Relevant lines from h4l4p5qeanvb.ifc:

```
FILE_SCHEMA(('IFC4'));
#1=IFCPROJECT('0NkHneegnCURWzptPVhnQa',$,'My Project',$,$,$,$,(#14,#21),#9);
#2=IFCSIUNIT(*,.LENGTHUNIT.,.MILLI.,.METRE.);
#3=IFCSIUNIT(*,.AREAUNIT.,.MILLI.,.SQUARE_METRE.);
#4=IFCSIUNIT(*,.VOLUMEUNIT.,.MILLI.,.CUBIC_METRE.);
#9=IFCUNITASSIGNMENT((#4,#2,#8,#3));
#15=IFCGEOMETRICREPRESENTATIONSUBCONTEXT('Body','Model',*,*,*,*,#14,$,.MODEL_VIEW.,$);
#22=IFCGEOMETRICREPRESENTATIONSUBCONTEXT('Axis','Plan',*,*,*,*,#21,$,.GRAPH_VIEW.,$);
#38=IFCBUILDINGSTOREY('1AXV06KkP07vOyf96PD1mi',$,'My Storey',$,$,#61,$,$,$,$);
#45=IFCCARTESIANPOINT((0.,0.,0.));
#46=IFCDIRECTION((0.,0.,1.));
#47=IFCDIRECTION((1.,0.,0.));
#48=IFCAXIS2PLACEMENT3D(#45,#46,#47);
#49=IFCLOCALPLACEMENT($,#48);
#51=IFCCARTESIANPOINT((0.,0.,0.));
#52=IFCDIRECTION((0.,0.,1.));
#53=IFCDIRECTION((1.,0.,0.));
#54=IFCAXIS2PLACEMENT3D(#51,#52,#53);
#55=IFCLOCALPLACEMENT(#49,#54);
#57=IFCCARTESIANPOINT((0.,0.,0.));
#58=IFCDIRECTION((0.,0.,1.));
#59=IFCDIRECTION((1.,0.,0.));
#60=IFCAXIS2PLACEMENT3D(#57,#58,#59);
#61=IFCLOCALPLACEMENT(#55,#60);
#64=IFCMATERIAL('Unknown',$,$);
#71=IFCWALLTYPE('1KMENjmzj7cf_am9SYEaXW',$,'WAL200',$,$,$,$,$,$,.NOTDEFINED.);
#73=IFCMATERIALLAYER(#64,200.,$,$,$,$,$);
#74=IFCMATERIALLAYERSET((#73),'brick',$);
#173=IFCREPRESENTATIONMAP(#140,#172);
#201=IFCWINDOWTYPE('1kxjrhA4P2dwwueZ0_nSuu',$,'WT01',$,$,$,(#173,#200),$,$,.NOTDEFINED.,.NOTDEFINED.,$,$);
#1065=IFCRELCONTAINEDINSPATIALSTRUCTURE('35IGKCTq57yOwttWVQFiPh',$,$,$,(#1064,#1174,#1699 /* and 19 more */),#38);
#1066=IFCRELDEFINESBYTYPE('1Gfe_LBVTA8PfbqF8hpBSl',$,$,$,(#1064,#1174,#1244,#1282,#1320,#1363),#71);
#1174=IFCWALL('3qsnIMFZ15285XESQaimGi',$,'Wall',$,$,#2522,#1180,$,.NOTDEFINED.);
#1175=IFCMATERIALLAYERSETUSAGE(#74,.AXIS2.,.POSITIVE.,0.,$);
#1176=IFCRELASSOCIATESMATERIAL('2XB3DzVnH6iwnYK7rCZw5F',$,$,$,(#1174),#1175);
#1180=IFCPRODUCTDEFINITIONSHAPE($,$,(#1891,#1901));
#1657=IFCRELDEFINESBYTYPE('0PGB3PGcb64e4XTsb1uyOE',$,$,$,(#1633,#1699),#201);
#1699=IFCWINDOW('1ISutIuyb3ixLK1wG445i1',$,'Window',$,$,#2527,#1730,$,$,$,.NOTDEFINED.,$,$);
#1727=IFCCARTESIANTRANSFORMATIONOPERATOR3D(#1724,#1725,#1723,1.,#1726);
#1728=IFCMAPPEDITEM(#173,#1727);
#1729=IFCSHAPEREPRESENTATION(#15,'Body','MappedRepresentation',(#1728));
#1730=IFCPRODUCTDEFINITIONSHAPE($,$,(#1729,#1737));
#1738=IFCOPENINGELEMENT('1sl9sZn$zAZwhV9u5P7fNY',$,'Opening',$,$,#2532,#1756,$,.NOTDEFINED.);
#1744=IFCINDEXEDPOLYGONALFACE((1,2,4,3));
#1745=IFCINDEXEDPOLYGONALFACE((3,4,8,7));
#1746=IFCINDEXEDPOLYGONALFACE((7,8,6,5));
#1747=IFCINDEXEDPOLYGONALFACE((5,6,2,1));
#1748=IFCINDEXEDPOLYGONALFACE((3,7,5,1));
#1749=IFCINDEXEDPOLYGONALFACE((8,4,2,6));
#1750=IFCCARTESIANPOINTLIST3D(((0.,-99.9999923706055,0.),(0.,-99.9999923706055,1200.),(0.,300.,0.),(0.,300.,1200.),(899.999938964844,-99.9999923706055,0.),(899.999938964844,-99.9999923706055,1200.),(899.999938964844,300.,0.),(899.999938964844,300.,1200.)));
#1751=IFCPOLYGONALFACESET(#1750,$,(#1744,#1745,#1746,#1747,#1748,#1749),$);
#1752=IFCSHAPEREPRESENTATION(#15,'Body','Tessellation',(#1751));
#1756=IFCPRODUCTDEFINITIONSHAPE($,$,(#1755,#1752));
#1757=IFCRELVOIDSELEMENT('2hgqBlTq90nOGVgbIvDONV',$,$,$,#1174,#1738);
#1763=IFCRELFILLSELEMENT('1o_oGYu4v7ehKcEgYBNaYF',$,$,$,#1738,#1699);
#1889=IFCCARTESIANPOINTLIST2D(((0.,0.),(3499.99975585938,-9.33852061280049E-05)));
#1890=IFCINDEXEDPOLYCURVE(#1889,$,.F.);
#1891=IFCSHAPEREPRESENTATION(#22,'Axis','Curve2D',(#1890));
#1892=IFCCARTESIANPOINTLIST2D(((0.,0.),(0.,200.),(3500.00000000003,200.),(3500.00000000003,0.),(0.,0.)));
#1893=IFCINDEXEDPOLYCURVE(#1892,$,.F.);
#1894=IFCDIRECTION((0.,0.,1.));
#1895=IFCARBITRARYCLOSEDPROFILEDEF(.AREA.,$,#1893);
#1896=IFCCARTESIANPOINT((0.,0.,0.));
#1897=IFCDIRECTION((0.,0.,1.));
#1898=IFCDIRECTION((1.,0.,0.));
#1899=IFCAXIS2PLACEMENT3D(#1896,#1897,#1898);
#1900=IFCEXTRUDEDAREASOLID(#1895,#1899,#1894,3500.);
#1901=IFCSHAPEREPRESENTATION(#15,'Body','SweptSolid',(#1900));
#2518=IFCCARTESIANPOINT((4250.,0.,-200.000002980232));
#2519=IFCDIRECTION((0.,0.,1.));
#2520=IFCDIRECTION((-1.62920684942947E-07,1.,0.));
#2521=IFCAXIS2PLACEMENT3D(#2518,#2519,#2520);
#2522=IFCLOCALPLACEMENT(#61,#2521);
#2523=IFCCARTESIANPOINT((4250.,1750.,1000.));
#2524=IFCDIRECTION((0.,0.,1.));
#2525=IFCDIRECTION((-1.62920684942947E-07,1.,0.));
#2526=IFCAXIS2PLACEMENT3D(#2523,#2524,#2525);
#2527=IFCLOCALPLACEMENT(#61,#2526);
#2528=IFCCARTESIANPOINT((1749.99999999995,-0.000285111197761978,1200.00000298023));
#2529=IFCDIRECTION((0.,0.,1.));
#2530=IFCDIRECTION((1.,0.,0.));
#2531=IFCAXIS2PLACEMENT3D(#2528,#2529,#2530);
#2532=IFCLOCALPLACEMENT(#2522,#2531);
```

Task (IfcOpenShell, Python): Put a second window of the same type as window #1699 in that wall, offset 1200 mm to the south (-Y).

```python
import ifcopenshell
import ifcopenshell.api.feature
import ifcopenshell.api.geometry
import ifcopenshell.api.root
import ifcopenshell.geom
import ifcopenshell.util.element
import ifcopenshell.util.placement
import ifcopenshell.util.shape

model = ifcopenshell.open("h4l4p5qeanvb.ifc")
settings = ifcopenshell.geom.settings()


def volume(element):
    """Net volume in cubic metres, openings subtracted."""
    shape = ifcopenshell.geom.create_shape(settings, element)
    return ifcopenshell.util.shape.get_volume(shape.geometry)


window = model.by_guid("1ISutIuyb3ixLK1wG445i1")
opening = window.FillsVoids[0].RelatingOpeningElement
wall = opening.VoidsElements[0].RelatingBuildingElement
before = volume(wall)
shift = ifcopenshell.util.placement.get_local_placement(wall.ObjectPlacement)[:3, 0] * -1200.0

# copy_class copies the void relationship, type, container and properties, but no geometry.
new_opening = ifcopenshell.api.root.copy_class(model, product=opening)
new_opening.Representation = ifcopenshell.util.element.copy_deep(
    model, opening.Representation, exclude=["IfcGeometricRepresentationContext", "IfcRepresentationMap"]
)
new_window = ifcopenshell.api.root.copy_class(model, product=window)
new_window.Representation = ifcopenshell.util.element.copy_deep(
    model, window.Representation, exclude=["IfcGeometricRepresentationContext", "IfcRepresentationMap"]
)
ifcopenshell.api.feature.add_filling(model, opening=new_opening, element=new_window)

for old, new in ((opening, new_opening), (window, new_window)):
    matrix = ifcopenshell.util.placement.get_local_placement(old.ObjectPlacement)
    matrix[:3, 3] += shift
    ifcopenshell.api.geometry.edit_object_placement(model, product=new, matrix=matrix, is_si=False)

after = volume(wall)

print(f"wall volume {before:.3f} -> {after:.3f} m3")

model.write("h4l4p5qeanvb_v2.ifc")
```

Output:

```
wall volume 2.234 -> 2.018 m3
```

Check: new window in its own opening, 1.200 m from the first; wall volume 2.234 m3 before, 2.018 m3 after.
